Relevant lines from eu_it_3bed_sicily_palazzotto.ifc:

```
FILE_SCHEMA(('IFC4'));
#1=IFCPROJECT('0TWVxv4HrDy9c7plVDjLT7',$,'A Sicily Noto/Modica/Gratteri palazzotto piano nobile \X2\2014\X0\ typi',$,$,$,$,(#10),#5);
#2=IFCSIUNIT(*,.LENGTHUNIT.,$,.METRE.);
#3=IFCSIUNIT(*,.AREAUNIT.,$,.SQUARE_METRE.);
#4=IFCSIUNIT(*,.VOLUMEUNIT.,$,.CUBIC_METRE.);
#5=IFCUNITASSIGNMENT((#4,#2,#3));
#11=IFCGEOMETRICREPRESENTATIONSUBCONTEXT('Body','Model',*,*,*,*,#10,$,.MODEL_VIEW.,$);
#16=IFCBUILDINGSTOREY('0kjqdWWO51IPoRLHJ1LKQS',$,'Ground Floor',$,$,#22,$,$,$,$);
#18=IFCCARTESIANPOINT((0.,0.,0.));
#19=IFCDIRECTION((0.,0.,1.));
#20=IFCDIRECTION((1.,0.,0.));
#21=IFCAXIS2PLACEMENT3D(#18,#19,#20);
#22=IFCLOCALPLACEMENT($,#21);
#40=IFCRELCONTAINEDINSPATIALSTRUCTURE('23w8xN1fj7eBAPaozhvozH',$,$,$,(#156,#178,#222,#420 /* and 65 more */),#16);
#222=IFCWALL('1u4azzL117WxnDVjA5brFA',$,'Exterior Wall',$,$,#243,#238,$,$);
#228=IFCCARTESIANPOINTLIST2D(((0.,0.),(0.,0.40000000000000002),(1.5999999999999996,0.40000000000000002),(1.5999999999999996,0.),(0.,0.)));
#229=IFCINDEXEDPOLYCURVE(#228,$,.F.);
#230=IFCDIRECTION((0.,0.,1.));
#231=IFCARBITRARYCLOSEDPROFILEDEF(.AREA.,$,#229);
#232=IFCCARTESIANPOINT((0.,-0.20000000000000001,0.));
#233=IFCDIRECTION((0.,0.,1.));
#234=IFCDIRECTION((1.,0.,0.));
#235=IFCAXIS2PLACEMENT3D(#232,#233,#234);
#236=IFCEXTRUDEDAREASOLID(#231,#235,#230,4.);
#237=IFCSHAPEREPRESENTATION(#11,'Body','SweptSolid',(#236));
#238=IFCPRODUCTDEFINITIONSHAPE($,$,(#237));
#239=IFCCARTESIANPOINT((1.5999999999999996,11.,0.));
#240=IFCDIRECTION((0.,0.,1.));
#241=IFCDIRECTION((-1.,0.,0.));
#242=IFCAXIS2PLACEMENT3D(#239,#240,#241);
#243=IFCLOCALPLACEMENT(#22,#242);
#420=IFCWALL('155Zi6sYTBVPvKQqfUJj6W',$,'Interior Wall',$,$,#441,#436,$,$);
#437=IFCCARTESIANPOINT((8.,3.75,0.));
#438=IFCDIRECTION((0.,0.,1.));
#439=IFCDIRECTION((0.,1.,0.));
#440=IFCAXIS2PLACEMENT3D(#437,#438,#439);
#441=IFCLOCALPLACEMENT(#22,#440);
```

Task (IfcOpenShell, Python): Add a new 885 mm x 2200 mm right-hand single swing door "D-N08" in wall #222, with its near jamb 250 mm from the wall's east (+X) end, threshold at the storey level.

```python
import numpy as np
import ifcopenshell
import ifcopenshell.api.feature
import ifcopenshell.api.geometry
import ifcopenshell.api.root
import ifcopenshell.api.spatial
import ifcopenshell.geom
import ifcopenshell.util.element
import ifcopenshell.util.placement
import ifcopenshell.util.representation
import ifcopenshell.util.shape
import ifcopenshell.util.unit

model = ifcopenshell.open("eu_it_3bed_sicily_palazzotto.ifc")
unit_scale = ifcopenshell.util.unit.calculate_unit_scale(model)
settings = ifcopenshell.geom.settings()


def volume(element):
    """Net volume in cubic metres, openings subtracted."""
    shape = ifcopenshell.geom.create_shape(settings, element)
    return ifcopenshell.util.shape.get_volume(shape.geometry)


wall = model.by_guid("1u4azzL117WxnDVjA5brFA")
storey = ifcopenshell.util.element.get_container(wall, ifc_class="IfcBuildingStorey")
context = ifcopenshell.util.representation.get_context(model, "Model", "Body", "MODEL_VIEW")
before = volume(wall)

width, height, from_end, sill = 0.885, 2.2, 0.25, 0.0  # metres

# The wall runs along its own X axis, and the end named is its -X end.
wall_shape = ifcopenshell.geom.create_shape(settings, wall)
x, y, z = ifcopenshell.util.shape.get_vertices(wall_shape.geometry).T
start = x.min() + from_end
face, thickness = float(y.min()), float(y.max() - y.min())
wall_matrix = ifcopenshell.util.placement.get_local_placement(wall.ObjectPlacement)
level = ifcopenshell.util.placement.get_local_placement(storey.ObjectPlacement)[2, 3]


def in_wall(x, y):
    """Placement at x, y metres in the wall's axes, at sill height."""
    matrix = wall_matrix.copy()
    matrix[:, 3] = wall_matrix @ np.array([x / unit_scale, y / unit_scale, 0.0, 1.0])
    matrix[2, 3] = level + sill / unit_scale
    return matrix


# Opening: a box that overshoots both wall faces by 50 mm.
opening = ifcopenshell.api.root.create_entity(model, ifc_class="IfcOpeningElement", predefined_type="OPENING")
box = ifcopenshell.api.geometry.add_wall_representation(
    model, context=context, length=width, height=height, thickness=thickness + 0.1
)
ifcopenshell.api.geometry.assign_representation(model, product=opening, representation=box)
ifcopenshell.api.geometry.edit_object_placement(model, product=opening, matrix=in_wall(start, face - 0.05), is_si=False)
ifcopenshell.api.feature.add_feature(model, feature=opening, element=wall)

door = ifcopenshell.api.root.create_entity(model, ifc_class="IfcDoor", name="D-N08", predefined_type="DOOR")
door.OverallWidth, door.OverallHeight = width / unit_scale, height / unit_scale
door.OperationType = "SINGLE_SWING_RIGHT"
body = ifcopenshell.api.geometry.add_door_representation(
    model,
    context=context,
    overall_width=door.OverallWidth,
    overall_height=door.OverallHeight,
    operation_type="SINGLE_SWING_RIGHT",
    lining_properties={"LiningDepth": thickness / unit_scale, "ThresholdDepth": thickness / unit_scale},
)
ifcopenshell.api.geometry.assign_representation(model, product=door, representation=body)
ifcopenshell.api.spatial.assign_container(model, products=[door], relating_structure=storey)
ifcopenshell.api.feature.add_filling(model, opening=opening, element=door)

# The lining spans the wall, so the door starts at the wall face.
ifcopenshell.api.geometry.edit_object_placement(model, product=door, matrix=in_wall(start, face), is_si=False)

after = volume(wall)

print(f"wall volume {before:.3f} -> {after:.3f} m3")

model.write("eu_it_3bed_sicily_palazzotto_edited.ifc")
```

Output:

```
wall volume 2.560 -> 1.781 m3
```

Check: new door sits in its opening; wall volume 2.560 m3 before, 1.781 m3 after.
